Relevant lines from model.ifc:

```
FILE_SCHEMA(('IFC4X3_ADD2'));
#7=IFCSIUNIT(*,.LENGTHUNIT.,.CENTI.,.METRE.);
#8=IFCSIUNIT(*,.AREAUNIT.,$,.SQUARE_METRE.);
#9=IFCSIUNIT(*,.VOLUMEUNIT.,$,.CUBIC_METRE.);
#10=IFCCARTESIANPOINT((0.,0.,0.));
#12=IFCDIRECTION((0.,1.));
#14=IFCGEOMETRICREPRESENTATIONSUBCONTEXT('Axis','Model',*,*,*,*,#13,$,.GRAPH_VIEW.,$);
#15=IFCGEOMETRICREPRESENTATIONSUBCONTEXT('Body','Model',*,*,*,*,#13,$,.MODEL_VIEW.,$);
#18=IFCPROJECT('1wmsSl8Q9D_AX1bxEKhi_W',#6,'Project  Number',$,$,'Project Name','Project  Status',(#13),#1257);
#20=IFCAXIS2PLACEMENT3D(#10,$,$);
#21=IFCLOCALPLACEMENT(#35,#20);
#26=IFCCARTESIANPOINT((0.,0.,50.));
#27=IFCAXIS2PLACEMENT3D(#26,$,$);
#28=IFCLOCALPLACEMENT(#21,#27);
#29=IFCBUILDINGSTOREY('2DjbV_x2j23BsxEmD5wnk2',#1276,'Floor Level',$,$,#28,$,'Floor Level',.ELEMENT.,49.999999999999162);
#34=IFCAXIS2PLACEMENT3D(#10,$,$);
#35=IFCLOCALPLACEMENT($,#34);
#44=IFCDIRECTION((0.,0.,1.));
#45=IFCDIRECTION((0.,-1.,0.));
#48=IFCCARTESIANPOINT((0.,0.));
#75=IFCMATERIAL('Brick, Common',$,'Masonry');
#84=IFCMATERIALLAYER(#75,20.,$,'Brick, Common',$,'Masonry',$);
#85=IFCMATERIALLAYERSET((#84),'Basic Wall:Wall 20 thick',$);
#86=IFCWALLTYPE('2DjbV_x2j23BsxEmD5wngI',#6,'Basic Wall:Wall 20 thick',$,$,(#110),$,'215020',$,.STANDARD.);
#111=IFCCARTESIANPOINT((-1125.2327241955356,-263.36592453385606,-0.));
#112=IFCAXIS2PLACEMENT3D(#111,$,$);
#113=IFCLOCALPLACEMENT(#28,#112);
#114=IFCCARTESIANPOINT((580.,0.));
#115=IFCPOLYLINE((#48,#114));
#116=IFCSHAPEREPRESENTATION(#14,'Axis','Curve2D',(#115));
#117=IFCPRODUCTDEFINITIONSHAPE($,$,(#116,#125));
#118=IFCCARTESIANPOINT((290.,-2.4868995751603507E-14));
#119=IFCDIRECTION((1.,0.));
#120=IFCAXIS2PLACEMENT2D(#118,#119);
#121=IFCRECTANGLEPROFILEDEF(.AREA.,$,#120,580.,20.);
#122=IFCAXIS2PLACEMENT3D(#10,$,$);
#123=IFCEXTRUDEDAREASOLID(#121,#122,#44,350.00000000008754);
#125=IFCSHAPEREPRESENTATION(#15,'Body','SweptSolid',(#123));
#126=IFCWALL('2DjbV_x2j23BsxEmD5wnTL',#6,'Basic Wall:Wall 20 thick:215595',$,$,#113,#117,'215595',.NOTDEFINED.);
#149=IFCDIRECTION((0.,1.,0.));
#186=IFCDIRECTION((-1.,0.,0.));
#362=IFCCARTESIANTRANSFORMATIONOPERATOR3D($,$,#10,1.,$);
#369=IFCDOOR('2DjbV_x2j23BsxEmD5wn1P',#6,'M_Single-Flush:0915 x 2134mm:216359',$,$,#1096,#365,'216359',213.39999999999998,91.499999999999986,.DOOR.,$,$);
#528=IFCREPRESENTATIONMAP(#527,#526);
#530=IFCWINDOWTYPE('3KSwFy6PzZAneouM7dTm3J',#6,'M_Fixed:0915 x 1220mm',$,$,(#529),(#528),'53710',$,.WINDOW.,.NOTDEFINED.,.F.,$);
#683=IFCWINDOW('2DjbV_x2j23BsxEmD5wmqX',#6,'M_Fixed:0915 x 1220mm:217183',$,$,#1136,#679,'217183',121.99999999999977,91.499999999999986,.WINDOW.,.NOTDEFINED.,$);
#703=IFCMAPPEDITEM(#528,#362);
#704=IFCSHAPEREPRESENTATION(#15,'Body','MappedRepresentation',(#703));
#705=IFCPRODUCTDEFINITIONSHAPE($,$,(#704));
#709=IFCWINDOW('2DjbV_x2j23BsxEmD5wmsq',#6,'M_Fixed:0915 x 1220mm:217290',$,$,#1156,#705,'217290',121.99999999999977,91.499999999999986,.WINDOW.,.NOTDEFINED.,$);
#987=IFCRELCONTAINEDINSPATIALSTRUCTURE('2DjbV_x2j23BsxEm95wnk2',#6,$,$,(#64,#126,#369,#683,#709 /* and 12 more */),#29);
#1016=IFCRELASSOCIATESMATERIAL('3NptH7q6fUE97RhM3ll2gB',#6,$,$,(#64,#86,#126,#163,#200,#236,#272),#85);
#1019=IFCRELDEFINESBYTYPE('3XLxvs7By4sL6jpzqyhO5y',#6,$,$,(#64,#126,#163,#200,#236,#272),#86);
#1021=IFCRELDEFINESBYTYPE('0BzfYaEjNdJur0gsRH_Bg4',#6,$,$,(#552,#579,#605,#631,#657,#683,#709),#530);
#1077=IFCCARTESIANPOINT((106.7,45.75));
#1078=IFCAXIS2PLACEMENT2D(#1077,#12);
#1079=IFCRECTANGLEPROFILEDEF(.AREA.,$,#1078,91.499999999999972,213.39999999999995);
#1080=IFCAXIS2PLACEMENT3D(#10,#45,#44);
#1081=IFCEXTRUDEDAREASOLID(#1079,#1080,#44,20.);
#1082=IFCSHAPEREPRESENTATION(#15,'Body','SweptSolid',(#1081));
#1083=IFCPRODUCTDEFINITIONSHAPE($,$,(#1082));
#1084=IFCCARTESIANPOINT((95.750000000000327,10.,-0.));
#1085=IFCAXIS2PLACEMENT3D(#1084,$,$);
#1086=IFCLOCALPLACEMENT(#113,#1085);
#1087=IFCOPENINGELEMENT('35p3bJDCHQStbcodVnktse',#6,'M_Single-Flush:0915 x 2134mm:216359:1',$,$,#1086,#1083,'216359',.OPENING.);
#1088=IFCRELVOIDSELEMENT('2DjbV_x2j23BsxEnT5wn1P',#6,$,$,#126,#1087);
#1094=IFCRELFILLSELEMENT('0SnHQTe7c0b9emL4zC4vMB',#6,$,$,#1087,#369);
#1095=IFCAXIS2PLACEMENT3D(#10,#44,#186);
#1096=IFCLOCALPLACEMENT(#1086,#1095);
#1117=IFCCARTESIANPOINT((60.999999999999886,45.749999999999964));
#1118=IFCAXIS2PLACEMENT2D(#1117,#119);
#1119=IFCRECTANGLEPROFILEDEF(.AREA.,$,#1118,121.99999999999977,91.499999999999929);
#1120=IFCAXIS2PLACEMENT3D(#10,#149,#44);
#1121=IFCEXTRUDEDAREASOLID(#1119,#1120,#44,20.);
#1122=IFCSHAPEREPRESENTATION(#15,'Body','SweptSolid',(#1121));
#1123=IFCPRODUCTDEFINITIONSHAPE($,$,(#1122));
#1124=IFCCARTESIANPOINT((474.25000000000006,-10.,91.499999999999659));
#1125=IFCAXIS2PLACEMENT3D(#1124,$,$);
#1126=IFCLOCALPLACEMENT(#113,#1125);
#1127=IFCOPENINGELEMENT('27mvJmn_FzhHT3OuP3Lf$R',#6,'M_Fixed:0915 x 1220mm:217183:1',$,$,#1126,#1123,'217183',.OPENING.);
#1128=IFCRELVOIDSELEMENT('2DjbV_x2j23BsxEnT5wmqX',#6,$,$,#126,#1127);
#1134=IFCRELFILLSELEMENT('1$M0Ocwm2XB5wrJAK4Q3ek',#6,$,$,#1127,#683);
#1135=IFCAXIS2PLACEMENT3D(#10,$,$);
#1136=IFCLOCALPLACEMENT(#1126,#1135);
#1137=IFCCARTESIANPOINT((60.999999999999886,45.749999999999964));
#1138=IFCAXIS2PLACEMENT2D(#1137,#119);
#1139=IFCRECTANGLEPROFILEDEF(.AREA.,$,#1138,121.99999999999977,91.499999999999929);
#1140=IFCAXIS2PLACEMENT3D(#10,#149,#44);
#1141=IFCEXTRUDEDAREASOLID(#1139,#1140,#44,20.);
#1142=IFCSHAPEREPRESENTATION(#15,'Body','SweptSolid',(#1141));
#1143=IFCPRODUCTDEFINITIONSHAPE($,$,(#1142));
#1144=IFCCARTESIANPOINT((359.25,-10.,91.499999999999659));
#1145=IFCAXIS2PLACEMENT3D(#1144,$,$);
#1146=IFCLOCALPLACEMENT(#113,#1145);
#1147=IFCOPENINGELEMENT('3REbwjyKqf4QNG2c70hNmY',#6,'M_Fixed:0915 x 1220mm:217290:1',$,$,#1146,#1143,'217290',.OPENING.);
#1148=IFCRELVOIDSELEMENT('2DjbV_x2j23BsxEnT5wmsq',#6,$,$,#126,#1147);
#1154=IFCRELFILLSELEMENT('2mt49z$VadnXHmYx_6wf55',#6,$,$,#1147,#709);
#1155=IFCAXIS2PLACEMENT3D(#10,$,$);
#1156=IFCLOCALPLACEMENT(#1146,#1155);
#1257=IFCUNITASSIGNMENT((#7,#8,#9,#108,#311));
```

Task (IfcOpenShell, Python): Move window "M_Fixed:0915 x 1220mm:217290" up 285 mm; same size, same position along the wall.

```python
import numpy as np
import ifcopenshell
import ifcopenshell.api.geometry
import ifcopenshell.util.placement
import ifcopenshell.util.unit

model = ifcopenshell.open("model.ifc")
unit_scale = ifcopenshell.util.unit.calculate_unit_scale(model)

window = model.by_guid("2DjbV_x2j23BsxEmD5wmsq")
opening = window.FillsVoids[0].RelatingOpeningElement
dz = 0.285 / unit_scale

shift = np.array([0.0, 0.0, dz])
# The window is placed relative to its opening, so it follows when the opening moves.
matrix = ifcopenshell.util.placement.get_local_placement(opening.ObjectPlacement)
matrix[:3, 3] += shift
ifcopenshell.api.geometry.edit_object_placement(
    model, product=opening, matrix=matrix, is_si=False, should_transform_children=True
)

print(f"moved by {dz * unit_scale:+.3f} m")

model.write("model-out.ifc")
```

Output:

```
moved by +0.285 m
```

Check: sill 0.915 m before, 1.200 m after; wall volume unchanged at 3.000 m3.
